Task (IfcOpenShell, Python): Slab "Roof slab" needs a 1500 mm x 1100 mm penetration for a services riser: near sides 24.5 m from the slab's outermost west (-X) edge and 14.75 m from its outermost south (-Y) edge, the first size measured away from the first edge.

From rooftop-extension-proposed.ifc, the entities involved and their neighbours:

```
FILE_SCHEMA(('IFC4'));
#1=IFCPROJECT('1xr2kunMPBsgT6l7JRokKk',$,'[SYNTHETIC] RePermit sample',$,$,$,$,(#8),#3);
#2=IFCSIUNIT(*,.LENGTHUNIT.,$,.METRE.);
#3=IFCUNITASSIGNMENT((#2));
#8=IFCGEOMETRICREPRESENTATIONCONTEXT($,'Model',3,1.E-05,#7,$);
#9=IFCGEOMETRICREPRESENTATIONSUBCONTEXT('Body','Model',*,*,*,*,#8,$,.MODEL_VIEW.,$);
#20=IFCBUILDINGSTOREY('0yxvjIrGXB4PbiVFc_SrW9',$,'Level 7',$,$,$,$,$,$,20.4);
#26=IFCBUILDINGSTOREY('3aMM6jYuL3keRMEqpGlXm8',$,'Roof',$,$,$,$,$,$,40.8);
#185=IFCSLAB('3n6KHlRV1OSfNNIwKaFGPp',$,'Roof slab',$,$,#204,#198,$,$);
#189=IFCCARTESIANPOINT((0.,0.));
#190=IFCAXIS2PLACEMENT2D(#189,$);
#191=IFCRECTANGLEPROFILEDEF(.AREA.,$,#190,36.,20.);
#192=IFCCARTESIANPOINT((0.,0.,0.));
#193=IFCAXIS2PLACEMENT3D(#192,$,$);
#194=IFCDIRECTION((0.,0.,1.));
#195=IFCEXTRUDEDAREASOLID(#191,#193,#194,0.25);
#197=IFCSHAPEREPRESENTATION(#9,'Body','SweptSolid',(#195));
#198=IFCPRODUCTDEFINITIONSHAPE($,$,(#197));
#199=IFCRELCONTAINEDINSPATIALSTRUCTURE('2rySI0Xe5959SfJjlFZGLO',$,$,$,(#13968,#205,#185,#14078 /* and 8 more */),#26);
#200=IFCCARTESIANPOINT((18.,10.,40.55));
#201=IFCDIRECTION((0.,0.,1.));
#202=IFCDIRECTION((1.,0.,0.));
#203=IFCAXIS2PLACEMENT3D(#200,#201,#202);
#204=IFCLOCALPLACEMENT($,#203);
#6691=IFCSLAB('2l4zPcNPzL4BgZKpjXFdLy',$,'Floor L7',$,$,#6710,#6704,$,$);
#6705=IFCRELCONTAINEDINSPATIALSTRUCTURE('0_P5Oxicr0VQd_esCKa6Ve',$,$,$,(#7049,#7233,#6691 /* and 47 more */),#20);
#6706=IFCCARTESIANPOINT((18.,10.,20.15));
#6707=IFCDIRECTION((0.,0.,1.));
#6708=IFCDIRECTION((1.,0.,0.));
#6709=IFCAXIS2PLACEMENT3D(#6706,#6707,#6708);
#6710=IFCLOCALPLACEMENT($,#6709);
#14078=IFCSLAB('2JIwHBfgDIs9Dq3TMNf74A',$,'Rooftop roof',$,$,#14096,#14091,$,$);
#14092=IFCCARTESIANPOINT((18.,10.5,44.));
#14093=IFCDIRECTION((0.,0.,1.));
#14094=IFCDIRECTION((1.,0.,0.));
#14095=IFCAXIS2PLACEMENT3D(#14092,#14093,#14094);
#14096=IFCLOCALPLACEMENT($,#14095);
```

```python
import numpy as np
import ifcopenshell
import ifcopenshell.api.feature
import ifcopenshell.api.geometry
import ifcopenshell.api.root
import ifcopenshell.geom
import ifcopenshell.util.placement
import ifcopenshell.util.representation
import ifcopenshell.util.shape
import ifcopenshell.util.unit

model = ifcopenshell.open("rooftop-extension-proposed.ifc")
unit_scale = ifcopenshell.util.unit.calculate_unit_scale(model)
settings = ifcopenshell.geom.settings()


def volume(element):
    """Net volume in cubic metres, openings subtracted."""
    shape = ifcopenshell.geom.create_shape(settings, element)
    return ifcopenshell.util.shape.get_volume(shape.geometry)


slab = model.by_id(185)
before = volume(slab)

# Extent in the slab's own axes, in metres. The edges named are its -X and -Y sides.
slab_shape = ifcopenshell.geom.create_shape(settings, slab)
vertices = ifcopenshell.util.shape.get_vertices(slab_shape.geometry)
x_min, y_min, bottom = vertices.min(axis=0)
top = vertices[:, 2].max()

opening = ifcopenshell.api.root.create_entity(model, ifc_class="IfcOpeningElement", name="Services riser opening", predefined_type="OPENING")
context = ifcopenshell.util.representation.get_context(model, "Model", "Body", "MODEL_VIEW")
width, depth = 1.5, 1.1
outline = [(0.0, 0.0), (width, 0.0), (width, depth), (0.0, depth), (0.0, 0.0)]
# Overshoot both faces by 50 mm so the cut is clean.
shape = ifcopenshell.api.geometry.add_slab_representation(
    model, context=context, depth=top - bottom + 0.1, polyline=outline
)
ifcopenshell.api.geometry.assign_representation(model, product=opening, representation=shape)

matrix = ifcopenshell.util.placement.get_local_placement(slab.ObjectPlacement)
matrix[:, 3] = matrix @ np.append(np.array([x_min + 24.5, y_min + 14.75, bottom - 0.05]) / unit_scale, 1.0)
ifcopenshell.api.geometry.edit_object_placement(model, product=opening, matrix=matrix, is_si=False)
ifcopenshell.api.feature.add_feature(model, feature=opening, element=slab)

after = volume(slab)

print(f"slab volume {before:.3f} -> {after:.3f} m3")

model.write("rooftop-extension-proposed_updated.ifc")
```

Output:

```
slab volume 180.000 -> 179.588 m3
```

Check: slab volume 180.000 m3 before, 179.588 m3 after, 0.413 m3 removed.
